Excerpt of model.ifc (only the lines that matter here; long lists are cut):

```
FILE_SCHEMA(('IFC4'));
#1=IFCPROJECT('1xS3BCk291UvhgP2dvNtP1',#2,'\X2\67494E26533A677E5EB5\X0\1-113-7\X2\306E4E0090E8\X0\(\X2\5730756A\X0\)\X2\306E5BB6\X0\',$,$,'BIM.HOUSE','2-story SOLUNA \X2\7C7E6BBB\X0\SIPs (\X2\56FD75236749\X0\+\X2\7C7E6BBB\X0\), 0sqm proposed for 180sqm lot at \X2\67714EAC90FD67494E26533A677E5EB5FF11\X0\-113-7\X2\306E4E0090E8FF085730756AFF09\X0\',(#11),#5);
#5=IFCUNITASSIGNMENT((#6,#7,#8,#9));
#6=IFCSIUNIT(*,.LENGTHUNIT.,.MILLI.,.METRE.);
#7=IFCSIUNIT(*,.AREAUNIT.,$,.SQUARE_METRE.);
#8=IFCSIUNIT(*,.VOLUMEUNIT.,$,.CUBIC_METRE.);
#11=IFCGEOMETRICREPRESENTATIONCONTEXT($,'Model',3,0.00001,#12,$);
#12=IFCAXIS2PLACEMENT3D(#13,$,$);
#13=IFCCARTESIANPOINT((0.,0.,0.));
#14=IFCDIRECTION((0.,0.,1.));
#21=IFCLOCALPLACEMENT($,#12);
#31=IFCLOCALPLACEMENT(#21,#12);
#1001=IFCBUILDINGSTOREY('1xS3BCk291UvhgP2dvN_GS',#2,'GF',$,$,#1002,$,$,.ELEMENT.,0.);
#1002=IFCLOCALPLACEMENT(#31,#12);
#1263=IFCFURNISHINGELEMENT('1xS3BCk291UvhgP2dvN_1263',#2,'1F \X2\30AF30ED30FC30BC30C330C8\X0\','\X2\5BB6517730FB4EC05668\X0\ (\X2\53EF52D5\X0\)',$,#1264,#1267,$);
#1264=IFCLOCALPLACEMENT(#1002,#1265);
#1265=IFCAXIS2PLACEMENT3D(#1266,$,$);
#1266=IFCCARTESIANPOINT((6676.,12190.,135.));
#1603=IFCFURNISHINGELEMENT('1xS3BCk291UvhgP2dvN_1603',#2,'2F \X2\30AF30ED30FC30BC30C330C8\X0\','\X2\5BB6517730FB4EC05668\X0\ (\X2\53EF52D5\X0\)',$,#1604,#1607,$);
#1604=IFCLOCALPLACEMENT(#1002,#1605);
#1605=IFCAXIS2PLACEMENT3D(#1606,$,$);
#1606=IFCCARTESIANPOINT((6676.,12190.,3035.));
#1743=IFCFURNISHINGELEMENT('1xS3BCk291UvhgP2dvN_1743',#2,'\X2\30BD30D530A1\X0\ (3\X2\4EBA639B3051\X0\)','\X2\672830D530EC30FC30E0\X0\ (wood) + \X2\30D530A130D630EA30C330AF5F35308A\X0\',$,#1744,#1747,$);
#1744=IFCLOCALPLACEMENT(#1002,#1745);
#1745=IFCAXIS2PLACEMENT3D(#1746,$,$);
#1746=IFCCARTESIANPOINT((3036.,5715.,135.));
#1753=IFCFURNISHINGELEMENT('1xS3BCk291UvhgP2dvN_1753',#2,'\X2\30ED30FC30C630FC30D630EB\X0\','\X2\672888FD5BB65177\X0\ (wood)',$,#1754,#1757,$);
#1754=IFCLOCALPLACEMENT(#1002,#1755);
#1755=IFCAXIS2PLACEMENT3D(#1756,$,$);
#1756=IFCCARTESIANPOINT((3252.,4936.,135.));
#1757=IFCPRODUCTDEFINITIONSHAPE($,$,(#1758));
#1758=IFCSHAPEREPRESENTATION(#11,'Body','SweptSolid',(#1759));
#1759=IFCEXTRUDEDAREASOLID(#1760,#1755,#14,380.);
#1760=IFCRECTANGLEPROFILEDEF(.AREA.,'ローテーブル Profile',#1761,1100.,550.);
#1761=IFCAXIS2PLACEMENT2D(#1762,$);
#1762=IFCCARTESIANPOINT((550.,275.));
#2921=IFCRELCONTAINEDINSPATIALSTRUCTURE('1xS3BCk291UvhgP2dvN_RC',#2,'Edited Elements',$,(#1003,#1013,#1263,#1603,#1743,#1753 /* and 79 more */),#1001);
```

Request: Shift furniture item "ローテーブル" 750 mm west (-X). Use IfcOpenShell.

```python
import ifcopenshell
import ifcopenshell.api.geometry
import ifcopenshell.util.placement
import ifcopenshell.util.unit

model = ifcopenshell.open("model.ifc")
unit_scale = ifcopenshell.util.unit.calculate_unit_scale(model)

item = model.by_id(1753)
matrix = ifcopenshell.util.placement.get_local_placement(item.ObjectPlacement)
matrix[0, 3] -= 0.75 / unit_scale
ifcopenshell.api.geometry.edit_object_placement(model, product=item, matrix=matrix, is_si=False)

print(ifcopenshell.util.placement.get_local_placement(item.ObjectPlacement).round(3) + 0.0)

model.write("model_rev.ifc")
```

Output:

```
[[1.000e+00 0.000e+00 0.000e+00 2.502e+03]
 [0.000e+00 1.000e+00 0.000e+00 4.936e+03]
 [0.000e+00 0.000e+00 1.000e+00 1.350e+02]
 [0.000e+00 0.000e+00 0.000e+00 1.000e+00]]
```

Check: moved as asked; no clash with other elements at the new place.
